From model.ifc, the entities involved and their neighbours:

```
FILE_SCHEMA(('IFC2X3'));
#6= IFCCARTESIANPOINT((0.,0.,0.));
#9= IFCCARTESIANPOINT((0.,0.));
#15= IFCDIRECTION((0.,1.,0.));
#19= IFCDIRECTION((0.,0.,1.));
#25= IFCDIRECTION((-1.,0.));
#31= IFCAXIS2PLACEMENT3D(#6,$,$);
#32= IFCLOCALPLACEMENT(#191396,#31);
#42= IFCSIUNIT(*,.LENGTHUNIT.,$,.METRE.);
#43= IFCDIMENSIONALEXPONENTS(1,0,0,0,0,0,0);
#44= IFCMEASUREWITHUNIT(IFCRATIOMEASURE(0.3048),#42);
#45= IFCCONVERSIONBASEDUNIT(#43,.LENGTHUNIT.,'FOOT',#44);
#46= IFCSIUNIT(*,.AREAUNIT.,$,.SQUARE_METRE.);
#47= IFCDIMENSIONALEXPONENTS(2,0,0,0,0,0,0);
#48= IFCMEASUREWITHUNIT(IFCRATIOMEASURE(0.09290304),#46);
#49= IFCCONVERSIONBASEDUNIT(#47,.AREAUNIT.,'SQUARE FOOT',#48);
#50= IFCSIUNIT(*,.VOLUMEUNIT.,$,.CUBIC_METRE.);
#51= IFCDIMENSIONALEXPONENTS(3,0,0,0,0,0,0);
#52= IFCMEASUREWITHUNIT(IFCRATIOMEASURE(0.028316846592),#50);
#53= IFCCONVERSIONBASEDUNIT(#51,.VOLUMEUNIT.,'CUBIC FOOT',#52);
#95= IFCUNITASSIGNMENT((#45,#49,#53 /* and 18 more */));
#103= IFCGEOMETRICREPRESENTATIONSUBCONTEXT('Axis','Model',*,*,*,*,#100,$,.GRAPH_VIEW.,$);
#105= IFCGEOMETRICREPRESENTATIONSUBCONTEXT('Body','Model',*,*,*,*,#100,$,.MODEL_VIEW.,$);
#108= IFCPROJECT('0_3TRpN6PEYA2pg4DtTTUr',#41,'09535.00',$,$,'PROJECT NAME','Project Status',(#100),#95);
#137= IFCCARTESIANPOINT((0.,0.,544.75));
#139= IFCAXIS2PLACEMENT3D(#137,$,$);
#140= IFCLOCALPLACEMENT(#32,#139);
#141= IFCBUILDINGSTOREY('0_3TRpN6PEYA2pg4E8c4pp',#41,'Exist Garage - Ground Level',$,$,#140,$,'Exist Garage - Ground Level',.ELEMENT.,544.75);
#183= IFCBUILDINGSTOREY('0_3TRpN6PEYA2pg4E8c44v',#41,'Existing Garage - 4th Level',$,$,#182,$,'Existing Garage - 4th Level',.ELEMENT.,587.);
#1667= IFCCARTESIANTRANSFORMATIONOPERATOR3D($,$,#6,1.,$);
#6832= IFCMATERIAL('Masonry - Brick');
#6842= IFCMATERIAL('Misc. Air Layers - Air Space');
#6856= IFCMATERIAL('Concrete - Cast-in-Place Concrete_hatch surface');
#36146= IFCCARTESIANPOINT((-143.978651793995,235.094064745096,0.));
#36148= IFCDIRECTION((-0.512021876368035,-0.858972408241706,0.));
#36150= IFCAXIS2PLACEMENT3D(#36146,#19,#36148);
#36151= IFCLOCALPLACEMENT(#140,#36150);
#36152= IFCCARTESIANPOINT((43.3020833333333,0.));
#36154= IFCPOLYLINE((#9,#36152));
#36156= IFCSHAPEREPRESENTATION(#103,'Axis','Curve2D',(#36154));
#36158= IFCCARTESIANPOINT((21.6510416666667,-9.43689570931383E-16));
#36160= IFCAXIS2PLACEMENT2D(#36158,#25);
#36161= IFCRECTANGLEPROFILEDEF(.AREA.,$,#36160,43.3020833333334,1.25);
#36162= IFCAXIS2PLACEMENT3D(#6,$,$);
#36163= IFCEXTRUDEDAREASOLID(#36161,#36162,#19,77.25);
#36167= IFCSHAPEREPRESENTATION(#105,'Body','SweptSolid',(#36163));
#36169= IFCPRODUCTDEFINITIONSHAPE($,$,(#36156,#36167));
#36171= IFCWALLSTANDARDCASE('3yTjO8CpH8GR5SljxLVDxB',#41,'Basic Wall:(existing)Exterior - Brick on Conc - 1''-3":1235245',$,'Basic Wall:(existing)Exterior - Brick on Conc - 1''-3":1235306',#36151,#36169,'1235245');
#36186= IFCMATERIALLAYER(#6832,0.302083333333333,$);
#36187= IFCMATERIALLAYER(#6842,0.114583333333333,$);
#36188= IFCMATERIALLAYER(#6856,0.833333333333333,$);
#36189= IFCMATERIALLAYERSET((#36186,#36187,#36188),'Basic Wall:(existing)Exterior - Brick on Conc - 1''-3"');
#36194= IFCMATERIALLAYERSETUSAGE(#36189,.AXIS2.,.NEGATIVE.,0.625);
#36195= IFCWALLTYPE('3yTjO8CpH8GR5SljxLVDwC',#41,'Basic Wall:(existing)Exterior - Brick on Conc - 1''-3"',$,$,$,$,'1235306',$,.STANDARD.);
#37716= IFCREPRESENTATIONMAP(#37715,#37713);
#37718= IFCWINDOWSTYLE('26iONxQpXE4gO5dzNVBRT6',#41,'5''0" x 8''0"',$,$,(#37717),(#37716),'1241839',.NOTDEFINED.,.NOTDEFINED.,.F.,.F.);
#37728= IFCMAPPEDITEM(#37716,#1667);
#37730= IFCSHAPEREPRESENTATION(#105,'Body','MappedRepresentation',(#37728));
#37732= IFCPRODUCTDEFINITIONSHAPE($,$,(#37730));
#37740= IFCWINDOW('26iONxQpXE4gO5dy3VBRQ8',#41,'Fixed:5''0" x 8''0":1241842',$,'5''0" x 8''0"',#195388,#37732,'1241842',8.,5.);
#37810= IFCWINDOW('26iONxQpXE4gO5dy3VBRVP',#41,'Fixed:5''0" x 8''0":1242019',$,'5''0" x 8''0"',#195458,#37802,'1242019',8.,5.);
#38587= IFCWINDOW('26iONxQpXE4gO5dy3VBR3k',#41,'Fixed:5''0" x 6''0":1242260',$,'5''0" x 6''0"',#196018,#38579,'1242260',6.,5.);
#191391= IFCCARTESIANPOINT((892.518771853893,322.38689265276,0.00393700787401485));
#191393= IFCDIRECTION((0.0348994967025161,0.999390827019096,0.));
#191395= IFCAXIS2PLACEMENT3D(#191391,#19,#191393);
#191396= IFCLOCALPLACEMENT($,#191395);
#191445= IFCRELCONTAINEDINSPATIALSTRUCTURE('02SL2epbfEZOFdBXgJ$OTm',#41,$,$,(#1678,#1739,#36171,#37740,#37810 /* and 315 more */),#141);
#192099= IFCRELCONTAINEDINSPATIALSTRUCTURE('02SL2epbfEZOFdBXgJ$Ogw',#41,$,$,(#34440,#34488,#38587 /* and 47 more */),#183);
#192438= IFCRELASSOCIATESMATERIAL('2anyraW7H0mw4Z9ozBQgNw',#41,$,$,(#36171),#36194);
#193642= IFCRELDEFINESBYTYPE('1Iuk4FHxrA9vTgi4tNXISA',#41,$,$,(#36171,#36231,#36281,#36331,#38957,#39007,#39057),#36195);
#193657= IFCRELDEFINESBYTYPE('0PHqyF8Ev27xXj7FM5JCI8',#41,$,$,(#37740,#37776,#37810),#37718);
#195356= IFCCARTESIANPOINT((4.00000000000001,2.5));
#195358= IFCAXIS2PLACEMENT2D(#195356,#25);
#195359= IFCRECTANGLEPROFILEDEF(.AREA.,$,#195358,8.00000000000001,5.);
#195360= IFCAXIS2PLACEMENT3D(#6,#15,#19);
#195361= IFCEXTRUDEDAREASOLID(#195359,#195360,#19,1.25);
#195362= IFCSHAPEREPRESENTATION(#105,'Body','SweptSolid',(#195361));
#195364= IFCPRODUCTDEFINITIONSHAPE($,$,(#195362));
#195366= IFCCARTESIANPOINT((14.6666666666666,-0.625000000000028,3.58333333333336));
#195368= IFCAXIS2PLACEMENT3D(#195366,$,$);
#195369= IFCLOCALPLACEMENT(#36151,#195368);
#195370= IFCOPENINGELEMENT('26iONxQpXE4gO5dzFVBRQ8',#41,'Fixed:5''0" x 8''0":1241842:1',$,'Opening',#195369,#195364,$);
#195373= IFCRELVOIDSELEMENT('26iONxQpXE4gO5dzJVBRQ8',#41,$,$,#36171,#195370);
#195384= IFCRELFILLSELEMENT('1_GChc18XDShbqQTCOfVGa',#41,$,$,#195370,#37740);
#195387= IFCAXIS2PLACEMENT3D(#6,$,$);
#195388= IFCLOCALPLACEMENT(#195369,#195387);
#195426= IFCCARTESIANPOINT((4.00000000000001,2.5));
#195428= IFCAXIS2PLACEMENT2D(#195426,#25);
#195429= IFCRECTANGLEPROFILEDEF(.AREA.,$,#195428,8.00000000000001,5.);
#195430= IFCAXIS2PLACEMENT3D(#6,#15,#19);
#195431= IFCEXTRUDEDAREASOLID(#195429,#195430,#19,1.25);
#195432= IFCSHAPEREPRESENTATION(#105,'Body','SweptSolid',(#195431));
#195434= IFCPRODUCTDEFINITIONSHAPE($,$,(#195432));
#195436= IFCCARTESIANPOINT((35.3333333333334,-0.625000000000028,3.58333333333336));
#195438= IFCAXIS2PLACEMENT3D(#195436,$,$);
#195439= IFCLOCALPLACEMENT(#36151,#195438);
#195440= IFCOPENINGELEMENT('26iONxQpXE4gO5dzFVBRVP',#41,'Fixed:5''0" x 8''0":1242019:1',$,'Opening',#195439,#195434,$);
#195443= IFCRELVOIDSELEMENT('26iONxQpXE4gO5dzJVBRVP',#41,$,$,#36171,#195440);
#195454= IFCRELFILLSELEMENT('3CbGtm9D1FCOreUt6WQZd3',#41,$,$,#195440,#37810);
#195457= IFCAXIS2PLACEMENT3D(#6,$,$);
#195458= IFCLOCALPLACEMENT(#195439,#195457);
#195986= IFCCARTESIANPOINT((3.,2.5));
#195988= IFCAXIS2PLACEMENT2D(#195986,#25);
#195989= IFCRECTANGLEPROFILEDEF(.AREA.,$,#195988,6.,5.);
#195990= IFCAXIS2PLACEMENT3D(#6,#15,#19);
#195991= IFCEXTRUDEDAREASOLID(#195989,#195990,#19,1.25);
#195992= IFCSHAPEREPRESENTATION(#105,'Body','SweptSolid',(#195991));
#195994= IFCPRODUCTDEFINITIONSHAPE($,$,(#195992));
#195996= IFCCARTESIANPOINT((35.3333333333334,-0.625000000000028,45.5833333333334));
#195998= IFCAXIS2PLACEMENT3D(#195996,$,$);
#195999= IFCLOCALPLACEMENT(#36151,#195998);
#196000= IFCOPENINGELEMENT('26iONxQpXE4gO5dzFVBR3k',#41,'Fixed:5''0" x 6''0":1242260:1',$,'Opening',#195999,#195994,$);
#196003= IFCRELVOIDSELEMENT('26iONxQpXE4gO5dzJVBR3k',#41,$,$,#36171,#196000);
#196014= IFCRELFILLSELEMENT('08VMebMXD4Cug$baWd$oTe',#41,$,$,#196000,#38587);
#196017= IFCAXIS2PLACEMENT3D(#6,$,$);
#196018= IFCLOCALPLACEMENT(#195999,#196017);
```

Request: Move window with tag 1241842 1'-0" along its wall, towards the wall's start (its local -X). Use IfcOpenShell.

```python
import ifcopenshell
import ifcopenshell.api.geometry
import ifcopenshell.util.placement
import ifcopenshell.util.unit

model = ifcopenshell.open("model.ifc")
unit_scale = ifcopenshell.util.unit.calculate_unit_scale(model)

window = model.by_id(37740)
opening = window.FillsVoids[0].RelatingOpeningElement
wall = opening.VoidsElements[0].RelatingBuildingElement

wall_matrix = ifcopenshell.util.placement.get_local_placement(wall.ObjectPlacement)
shift = wall_matrix[:3, 0] * -12 * 0.0254 / unit_scale
before = ifcopenshell.util.placement.get_local_placement(window.ObjectPlacement)[:3, 3].copy()

# The window is placed relative to its opening, so it follows when the opening moves.
matrix = ifcopenshell.util.placement.get_local_placement(opening.ObjectPlacement)
matrix[:3, 3] += shift
ifcopenshell.api.geometry.edit_object_placement(
    model, product=opening, matrix=matrix, is_si=False, should_transform_children=True
)

after = ifcopenshell.util.placement.get_local_placement(window.ObjectPlacement)[:3, 3]
print("window moved by", (after - before).round(3) + 0.0)

model.write("model_rev.ifc")
```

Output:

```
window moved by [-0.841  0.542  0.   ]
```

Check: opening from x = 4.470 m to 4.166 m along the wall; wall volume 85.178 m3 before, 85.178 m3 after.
